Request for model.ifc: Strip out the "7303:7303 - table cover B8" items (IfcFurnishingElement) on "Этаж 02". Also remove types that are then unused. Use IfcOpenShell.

First a look at what the model holds.

```python
import ifcopenshell
import ifcopenshell.util.element

model = ifcopenshell.open("model.ifc")
print(model.schema)
storey = next(s for s in model.by_type("IfcBuildingStorey") if s.Name == "Этаж 02")
furniture = [e for e in ifcopenshell.util.element.get_decomposition(storey) if e.is_a("IfcFurnishingElement")]
seen = {}
for e in furniture:
    element_type = ifcopenshell.util.element.get_type(e)
    name = element_type.Name if element_type not in (None, e) else None
    seen[name] = seen.get(name, 0) + 1
for name, count in sorted(seen.items(), key=str):
    print(count, "x", name)
```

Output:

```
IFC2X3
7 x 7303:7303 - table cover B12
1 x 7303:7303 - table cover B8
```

```python
import ifcopenshell
import ifcopenshell.api.root
import ifcopenshell.util.element

model = ifcopenshell.open("model.ifc")

storey = next(s for s in model.by_type("IfcBuildingStorey") if s.Name == "Этаж 02")
furniture = [e for e in ifcopenshell.util.element.get_decomposition(storey) if e.is_a("IfcFurnishingElement")]
targets = [e for e in furniture if (t := ifcopenshell.util.element.get_type(e)) not in (None, e) and t.Name == "7303:7303 - table cover B8"]
types = {ifcopenshell.util.element.get_type(e) for e in targets} - {None, *targets}

for e in targets:
    ifcopenshell.api.root.remove_product(model, product=e)
print(len(targets), "removed")

unused = [t for t in types if not ifcopenshell.util.element.get_types(t)]
for t in unused:
    ifcopenshell.api.root.remove_product(model, product=t)
print(len(unused), "unused types removed")

model.write("model_rev.ifc")
```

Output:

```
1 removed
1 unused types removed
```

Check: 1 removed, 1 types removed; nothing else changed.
